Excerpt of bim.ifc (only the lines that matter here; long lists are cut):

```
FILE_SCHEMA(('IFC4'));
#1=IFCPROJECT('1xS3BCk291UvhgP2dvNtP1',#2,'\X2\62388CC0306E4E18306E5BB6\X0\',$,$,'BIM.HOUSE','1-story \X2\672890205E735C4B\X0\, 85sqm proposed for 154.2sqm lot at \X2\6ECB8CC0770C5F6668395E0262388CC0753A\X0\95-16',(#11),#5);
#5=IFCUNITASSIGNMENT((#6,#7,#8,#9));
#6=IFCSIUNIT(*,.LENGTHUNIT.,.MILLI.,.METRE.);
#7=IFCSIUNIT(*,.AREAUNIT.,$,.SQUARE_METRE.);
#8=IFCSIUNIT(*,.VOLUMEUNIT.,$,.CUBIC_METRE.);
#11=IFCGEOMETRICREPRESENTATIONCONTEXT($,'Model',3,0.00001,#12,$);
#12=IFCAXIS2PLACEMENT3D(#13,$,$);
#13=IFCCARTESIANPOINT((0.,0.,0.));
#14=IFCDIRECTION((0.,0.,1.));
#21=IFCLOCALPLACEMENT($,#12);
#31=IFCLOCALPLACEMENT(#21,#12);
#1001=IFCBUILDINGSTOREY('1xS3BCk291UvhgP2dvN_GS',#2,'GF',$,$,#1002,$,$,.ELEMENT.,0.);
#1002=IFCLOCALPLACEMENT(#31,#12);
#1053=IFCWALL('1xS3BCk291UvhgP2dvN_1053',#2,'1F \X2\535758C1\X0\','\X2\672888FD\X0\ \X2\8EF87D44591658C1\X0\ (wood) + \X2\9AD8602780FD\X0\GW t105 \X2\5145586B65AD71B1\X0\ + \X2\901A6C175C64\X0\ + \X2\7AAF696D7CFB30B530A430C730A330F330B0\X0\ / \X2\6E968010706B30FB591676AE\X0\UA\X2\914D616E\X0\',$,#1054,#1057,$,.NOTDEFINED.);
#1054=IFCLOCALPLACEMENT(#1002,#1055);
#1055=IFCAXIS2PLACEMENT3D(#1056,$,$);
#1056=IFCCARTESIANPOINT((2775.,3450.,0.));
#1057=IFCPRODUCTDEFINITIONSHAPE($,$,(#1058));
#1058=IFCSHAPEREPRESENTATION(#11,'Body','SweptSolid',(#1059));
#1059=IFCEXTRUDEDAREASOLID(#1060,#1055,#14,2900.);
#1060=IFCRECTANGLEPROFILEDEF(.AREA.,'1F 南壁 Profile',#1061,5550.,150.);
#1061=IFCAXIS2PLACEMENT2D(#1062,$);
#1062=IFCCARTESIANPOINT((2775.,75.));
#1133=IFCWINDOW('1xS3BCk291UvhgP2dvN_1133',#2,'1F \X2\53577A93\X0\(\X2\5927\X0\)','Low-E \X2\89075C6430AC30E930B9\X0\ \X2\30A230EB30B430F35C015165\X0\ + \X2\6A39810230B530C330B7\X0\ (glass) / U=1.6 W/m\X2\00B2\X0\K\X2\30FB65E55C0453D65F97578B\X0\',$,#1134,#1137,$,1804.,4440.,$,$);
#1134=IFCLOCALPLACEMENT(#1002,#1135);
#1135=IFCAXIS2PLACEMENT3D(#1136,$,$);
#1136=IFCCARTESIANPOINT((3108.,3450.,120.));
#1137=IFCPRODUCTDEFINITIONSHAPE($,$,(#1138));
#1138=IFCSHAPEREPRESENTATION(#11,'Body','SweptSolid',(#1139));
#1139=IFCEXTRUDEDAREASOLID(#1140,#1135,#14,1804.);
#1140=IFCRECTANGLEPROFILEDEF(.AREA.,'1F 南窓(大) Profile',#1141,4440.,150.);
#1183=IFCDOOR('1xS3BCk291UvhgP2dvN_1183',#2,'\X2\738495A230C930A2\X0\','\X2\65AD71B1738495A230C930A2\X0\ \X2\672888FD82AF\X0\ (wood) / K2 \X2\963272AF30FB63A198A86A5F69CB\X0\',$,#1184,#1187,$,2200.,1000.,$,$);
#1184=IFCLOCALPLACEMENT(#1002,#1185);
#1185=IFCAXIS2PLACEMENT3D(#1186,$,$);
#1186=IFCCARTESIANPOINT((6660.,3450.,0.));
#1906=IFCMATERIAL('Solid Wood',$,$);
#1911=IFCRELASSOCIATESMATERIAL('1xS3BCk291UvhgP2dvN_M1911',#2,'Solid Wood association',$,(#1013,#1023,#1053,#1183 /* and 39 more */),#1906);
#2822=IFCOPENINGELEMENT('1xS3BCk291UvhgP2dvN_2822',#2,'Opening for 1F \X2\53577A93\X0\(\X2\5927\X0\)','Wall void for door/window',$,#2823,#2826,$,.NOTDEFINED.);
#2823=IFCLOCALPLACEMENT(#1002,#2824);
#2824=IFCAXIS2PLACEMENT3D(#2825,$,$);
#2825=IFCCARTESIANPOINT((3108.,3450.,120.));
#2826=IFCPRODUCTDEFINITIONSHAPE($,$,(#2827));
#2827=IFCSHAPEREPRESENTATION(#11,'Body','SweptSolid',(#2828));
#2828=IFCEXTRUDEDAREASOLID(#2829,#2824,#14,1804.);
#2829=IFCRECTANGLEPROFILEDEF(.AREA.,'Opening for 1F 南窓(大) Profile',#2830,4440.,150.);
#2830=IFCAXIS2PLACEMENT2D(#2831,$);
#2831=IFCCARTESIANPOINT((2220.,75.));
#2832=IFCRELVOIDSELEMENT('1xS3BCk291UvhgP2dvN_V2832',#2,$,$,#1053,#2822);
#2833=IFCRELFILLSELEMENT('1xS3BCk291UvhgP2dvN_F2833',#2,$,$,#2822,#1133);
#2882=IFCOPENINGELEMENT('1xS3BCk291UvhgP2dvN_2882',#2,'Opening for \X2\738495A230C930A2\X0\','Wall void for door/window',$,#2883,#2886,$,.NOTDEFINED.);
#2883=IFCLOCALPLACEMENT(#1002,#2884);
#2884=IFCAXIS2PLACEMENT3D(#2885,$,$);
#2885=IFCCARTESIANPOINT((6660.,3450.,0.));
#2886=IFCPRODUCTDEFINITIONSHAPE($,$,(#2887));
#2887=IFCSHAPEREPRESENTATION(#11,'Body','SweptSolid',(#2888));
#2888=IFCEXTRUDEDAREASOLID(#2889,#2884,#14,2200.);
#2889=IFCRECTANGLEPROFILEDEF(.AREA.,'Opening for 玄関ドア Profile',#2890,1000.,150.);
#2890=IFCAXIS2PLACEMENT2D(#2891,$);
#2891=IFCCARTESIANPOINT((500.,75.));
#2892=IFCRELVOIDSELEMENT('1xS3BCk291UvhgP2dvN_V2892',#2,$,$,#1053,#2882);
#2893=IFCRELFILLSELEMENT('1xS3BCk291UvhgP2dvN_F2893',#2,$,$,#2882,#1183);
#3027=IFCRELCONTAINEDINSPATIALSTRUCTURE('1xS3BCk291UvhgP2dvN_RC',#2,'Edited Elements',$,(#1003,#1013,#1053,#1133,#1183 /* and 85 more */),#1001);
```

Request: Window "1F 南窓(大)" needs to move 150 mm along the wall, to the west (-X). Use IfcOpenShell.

```python
import ifcopenshell
import ifcopenshell.api.geometry
import ifcopenshell.util.placement
import ifcopenshell.util.unit

model = ifcopenshell.open("bim.ifc")
unit_scale = ifcopenshell.util.unit.calculate_unit_scale(model)

window = model.by_guid("1xS3BCk291UvhgP2dvN_1133")
opening = window.FillsVoids[0].RelatingOpeningElement
wall = opening.VoidsElements[0].RelatingBuildingElement

wall_matrix = ifcopenshell.util.placement.get_local_placement(wall.ObjectPlacement)
shift = wall_matrix[:3, 0] * -0.15 / unit_scale
before = ifcopenshell.util.placement.get_local_placement(window.ObjectPlacement)[:3, 3].copy()

# The window is not placed relative to its opening, so move both.
for product in (opening, window):
    matrix = ifcopenshell.util.placement.get_local_placement(product.ObjectPlacement)
    matrix[:3, 3] += shift
    ifcopenshell.api.geometry.edit_object_placement(model, product=product, matrix=matrix, is_si=False)

after = ifcopenshell.util.placement.get_local_placement(window.ObjectPlacement)[:3, 3]
print("window moved by", (after - before).round(3) + 0.0)

model.write("bim_v2.ifc")
```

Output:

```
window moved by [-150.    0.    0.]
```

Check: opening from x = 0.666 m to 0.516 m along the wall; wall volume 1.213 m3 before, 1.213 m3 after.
